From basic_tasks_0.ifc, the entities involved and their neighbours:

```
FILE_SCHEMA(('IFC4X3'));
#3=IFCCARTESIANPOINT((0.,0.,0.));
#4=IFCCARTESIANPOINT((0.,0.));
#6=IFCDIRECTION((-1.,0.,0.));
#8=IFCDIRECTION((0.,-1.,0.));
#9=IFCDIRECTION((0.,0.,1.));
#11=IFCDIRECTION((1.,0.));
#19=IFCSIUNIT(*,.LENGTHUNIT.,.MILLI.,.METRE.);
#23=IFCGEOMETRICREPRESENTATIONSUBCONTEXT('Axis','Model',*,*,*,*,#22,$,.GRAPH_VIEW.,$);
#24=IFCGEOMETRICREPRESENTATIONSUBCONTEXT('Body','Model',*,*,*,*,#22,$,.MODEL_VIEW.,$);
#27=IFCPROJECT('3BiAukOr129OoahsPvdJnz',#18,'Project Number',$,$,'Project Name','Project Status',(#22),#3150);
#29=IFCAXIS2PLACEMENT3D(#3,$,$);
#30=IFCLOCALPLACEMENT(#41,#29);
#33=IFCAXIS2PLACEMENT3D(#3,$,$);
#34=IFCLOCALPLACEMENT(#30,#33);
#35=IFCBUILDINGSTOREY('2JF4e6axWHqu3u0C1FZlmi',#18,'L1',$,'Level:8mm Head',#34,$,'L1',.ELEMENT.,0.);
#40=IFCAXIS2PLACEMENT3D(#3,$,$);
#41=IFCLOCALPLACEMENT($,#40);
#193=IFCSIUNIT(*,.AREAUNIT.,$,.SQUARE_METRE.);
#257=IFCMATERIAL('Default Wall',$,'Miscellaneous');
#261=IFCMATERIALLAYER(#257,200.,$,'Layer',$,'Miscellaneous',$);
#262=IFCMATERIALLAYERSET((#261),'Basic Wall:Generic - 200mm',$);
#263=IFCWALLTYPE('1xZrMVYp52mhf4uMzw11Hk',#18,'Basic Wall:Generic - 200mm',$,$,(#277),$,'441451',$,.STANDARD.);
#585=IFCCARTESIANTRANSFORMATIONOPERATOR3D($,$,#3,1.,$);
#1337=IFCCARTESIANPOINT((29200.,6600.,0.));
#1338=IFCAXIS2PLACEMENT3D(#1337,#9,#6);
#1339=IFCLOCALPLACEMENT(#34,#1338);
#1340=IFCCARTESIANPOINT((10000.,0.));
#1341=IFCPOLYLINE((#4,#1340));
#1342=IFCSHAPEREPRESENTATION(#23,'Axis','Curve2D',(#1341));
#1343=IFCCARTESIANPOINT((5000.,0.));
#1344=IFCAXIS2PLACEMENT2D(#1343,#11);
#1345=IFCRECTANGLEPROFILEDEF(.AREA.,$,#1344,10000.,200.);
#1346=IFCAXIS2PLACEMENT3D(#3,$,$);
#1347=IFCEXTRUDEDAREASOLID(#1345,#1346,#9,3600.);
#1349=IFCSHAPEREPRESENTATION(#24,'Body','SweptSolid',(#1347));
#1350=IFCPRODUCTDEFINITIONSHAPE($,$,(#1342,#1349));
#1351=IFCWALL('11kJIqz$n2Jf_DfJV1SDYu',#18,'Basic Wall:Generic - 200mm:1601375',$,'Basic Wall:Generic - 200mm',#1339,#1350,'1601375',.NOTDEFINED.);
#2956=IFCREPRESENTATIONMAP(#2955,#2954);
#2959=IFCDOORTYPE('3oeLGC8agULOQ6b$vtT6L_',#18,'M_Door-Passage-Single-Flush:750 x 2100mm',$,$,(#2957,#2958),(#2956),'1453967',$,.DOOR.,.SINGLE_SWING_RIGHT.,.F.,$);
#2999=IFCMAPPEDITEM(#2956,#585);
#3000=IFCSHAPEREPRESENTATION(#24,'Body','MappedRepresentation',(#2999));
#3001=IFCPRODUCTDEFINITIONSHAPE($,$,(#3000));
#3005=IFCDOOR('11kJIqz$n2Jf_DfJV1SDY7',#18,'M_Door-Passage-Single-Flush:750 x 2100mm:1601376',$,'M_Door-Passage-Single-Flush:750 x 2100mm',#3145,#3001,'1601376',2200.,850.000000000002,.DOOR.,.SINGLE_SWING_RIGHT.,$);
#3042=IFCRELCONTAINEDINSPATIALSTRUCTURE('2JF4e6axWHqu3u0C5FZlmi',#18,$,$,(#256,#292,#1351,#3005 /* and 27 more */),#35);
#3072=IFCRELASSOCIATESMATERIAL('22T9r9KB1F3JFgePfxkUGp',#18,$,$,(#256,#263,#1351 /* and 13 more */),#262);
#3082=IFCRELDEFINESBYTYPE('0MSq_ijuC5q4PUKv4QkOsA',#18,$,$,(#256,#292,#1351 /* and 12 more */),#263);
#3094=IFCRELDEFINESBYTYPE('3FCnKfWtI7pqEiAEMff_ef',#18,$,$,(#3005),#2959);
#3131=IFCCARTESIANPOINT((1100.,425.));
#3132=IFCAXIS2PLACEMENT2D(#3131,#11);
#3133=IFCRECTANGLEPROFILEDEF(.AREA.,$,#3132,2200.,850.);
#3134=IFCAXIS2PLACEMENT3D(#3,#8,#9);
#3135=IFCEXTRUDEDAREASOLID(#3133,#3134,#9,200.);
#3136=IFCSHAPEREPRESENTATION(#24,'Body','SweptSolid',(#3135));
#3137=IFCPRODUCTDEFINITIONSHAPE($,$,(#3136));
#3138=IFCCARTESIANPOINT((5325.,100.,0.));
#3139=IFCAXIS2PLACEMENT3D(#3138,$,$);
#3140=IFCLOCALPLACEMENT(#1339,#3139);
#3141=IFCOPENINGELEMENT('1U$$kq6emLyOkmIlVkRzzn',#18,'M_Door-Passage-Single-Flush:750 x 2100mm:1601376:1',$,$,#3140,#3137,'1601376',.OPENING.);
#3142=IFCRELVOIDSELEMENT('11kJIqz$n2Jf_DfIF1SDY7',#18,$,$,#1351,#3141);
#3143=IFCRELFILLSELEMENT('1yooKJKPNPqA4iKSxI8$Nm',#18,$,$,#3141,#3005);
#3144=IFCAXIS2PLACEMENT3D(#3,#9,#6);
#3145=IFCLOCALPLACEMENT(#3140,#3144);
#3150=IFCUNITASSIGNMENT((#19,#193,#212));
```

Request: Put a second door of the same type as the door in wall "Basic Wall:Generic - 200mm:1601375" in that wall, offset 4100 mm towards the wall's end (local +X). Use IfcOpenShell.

```python
import ifcopenshell
import ifcopenshell.api.feature
import ifcopenshell.api.geometry
import ifcopenshell.api.root
import ifcopenshell.geom
import ifcopenshell.util.element
import ifcopenshell.util.placement
import ifcopenshell.util.shape
import ifcopenshell.util.unit

model = ifcopenshell.open("basic_tasks_0.ifc")
unit_scale = ifcopenshell.util.unit.calculate_unit_scale(model)
settings = ifcopenshell.geom.settings()


def volume(element):
    """Net volume in cubic metres, openings subtracted."""
    shape = ifcopenshell.geom.create_shape(settings, element)
    return ifcopenshell.util.shape.get_volume(shape.geometry)


def reuse_history(source, copy):
    """copy_class also copies each property set's owner history, people and application; keep the originals."""
    for rel in copy.IsDefinedBy:
        if rel.is_a("IfcRelDefinesByProperties") and (history := rel.RelatingPropertyDefinition.OwnerHistory):
            rel.RelatingPropertyDefinition.OwnerHistory = source.OwnerHistory
            ifcopenshell.util.element.remove_deep2(model, history)


door = model.by_guid("11kJIqz$n2Jf_DfJV1SDY7")
opening = door.FillsVoids[0].RelatingOpeningElement
wall = opening.VoidsElements[0].RelatingBuildingElement
before = volume(wall)
shift = ifcopenshell.util.placement.get_local_placement(wall.ObjectPlacement)[:3, 0] * 4.1 / unit_scale

# copy_class copies the void relationship, type, container and properties, but no geometry.
new_opening = ifcopenshell.api.root.copy_class(model, product=opening)
new_opening.Representation = ifcopenshell.util.element.copy_deep(
    model, opening.Representation, exclude=["IfcGeometricRepresentationContext", "IfcRepresentationMap"]
)
new_opening.Name = "M_Door-Passage-Single-Flush:750 x 2100mm"
new_opening.Tag = None
new_door = ifcopenshell.api.root.copy_class(model, product=door)
new_door.Representation = ifcopenshell.util.element.copy_deep(
    model, door.Representation, exclude=["IfcGeometricRepresentationContext", "IfcRepresentationMap"]
)
new_door.Name = "M_Door-Passage-Single-Flush:750 x 2100mm"
new_door.Tag = None
reuse_history(door, new_door)
ifcopenshell.api.feature.add_filling(model, opening=new_opening, element=new_door)

for old, new in ((opening, new_opening), (door, new_door)):
    matrix = ifcopenshell.util.placement.get_local_placement(old.ObjectPlacement)
    matrix[:3, 3] += shift
    ifcopenshell.api.geometry.edit_object_placement(model, product=new, matrix=matrix, is_si=False)

after = volume(wall)

print(f"wall volume {before:.3f} -> {after:.3f} m3")

model.write("basic_tasks_0_v2.ifc")
```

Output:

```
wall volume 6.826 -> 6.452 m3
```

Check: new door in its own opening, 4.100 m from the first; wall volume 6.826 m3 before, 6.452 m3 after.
